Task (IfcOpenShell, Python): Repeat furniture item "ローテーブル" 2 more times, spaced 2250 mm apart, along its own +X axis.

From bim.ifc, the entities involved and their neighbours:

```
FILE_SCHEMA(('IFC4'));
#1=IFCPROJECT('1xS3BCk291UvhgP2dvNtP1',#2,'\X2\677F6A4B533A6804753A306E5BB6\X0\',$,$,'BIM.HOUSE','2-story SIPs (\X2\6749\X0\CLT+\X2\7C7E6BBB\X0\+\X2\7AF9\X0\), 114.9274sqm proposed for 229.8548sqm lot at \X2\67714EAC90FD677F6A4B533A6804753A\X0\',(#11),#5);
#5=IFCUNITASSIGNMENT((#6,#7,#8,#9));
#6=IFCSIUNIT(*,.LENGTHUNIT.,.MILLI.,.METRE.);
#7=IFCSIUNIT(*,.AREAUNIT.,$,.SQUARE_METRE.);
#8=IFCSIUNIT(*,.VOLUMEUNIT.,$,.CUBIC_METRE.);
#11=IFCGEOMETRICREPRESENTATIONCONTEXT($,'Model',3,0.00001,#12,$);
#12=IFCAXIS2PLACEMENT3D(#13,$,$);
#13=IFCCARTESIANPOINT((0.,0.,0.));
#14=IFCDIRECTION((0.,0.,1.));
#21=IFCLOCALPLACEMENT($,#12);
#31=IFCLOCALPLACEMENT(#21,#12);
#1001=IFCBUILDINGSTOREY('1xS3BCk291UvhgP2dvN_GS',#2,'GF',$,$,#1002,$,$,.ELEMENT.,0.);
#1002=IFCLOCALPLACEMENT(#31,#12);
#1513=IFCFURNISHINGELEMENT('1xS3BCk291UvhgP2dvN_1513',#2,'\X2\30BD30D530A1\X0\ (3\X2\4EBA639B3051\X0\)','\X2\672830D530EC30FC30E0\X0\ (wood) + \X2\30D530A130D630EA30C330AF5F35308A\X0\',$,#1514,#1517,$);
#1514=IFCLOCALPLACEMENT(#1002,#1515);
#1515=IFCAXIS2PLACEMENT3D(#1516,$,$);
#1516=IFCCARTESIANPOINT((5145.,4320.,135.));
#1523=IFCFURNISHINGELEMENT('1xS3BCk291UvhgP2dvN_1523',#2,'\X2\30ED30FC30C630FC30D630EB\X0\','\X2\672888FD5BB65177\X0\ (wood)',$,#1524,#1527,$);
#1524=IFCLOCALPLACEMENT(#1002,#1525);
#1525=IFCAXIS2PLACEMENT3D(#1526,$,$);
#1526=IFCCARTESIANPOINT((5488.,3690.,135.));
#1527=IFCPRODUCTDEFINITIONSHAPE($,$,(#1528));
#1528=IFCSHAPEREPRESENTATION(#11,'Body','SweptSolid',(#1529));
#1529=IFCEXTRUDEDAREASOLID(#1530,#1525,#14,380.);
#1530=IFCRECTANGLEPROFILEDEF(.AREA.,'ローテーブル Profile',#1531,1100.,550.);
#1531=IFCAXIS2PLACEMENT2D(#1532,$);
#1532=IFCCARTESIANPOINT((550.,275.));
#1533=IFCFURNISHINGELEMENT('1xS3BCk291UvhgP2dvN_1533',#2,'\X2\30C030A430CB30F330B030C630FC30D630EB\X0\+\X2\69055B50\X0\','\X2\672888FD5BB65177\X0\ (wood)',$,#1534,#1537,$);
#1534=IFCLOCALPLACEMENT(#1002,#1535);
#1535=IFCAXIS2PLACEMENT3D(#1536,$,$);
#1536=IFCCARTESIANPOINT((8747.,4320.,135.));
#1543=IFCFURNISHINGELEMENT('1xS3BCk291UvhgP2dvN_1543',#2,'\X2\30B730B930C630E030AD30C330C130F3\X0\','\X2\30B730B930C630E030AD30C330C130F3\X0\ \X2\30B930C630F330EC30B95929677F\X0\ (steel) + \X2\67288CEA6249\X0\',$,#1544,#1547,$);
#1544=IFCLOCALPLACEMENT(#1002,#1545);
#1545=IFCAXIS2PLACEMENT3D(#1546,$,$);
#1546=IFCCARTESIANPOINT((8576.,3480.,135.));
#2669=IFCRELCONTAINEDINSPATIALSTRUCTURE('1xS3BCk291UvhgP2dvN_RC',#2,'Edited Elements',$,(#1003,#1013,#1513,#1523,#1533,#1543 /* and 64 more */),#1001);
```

```python
import ifcopenshell
import ifcopenshell.api.geometry
import ifcopenshell.api.root
import ifcopenshell.util.element
import ifcopenshell.util.placement
import ifcopenshell.util.unit

model = ifcopenshell.open("bim.ifc")
unit_scale = ifcopenshell.util.unit.calculate_unit_scale(model)


def reuse_history(source, copy):
    """copy_class also copies each property set's owner history, people and application; keep the originals."""
    for rel in copy.IsDefinedBy:
        if rel.is_a("IfcRelDefinesByProperties") and (history := rel.RelatingPropertyDefinition.OwnerHistory):
            rel.RelatingPropertyDefinition.OwnerHistory = source.OwnerHistory
            ifcopenshell.util.element.remove_deep2(model, history)


source = model.by_guid("1xS3BCk291UvhgP2dvN_1523")
base = ifcopenshell.util.placement.get_local_placement(source.ObjectPlacement)
step = base[:3, 0] * 2.25 / unit_scale

for i in range(1, 3):
    copy = ifcopenshell.api.root.copy_class(model, product=source)
    copy.Representation = ifcopenshell.util.element.copy_deep(
        model, source.Representation, exclude=["IfcGeometricRepresentationContext", "IfcRepresentationMap"]
    )
    reuse_history(source, copy)
    matrix = base.copy()
    matrix[:3, 3] += i * step
    print("added at", matrix[:3, 3].round(3) + 0.0)
    ifcopenshell.api.geometry.edit_object_placement(model, product=copy, matrix=matrix, is_si=False)

model.write("bim_updated.ifc")
```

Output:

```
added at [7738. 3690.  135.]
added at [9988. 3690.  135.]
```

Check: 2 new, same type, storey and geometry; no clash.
